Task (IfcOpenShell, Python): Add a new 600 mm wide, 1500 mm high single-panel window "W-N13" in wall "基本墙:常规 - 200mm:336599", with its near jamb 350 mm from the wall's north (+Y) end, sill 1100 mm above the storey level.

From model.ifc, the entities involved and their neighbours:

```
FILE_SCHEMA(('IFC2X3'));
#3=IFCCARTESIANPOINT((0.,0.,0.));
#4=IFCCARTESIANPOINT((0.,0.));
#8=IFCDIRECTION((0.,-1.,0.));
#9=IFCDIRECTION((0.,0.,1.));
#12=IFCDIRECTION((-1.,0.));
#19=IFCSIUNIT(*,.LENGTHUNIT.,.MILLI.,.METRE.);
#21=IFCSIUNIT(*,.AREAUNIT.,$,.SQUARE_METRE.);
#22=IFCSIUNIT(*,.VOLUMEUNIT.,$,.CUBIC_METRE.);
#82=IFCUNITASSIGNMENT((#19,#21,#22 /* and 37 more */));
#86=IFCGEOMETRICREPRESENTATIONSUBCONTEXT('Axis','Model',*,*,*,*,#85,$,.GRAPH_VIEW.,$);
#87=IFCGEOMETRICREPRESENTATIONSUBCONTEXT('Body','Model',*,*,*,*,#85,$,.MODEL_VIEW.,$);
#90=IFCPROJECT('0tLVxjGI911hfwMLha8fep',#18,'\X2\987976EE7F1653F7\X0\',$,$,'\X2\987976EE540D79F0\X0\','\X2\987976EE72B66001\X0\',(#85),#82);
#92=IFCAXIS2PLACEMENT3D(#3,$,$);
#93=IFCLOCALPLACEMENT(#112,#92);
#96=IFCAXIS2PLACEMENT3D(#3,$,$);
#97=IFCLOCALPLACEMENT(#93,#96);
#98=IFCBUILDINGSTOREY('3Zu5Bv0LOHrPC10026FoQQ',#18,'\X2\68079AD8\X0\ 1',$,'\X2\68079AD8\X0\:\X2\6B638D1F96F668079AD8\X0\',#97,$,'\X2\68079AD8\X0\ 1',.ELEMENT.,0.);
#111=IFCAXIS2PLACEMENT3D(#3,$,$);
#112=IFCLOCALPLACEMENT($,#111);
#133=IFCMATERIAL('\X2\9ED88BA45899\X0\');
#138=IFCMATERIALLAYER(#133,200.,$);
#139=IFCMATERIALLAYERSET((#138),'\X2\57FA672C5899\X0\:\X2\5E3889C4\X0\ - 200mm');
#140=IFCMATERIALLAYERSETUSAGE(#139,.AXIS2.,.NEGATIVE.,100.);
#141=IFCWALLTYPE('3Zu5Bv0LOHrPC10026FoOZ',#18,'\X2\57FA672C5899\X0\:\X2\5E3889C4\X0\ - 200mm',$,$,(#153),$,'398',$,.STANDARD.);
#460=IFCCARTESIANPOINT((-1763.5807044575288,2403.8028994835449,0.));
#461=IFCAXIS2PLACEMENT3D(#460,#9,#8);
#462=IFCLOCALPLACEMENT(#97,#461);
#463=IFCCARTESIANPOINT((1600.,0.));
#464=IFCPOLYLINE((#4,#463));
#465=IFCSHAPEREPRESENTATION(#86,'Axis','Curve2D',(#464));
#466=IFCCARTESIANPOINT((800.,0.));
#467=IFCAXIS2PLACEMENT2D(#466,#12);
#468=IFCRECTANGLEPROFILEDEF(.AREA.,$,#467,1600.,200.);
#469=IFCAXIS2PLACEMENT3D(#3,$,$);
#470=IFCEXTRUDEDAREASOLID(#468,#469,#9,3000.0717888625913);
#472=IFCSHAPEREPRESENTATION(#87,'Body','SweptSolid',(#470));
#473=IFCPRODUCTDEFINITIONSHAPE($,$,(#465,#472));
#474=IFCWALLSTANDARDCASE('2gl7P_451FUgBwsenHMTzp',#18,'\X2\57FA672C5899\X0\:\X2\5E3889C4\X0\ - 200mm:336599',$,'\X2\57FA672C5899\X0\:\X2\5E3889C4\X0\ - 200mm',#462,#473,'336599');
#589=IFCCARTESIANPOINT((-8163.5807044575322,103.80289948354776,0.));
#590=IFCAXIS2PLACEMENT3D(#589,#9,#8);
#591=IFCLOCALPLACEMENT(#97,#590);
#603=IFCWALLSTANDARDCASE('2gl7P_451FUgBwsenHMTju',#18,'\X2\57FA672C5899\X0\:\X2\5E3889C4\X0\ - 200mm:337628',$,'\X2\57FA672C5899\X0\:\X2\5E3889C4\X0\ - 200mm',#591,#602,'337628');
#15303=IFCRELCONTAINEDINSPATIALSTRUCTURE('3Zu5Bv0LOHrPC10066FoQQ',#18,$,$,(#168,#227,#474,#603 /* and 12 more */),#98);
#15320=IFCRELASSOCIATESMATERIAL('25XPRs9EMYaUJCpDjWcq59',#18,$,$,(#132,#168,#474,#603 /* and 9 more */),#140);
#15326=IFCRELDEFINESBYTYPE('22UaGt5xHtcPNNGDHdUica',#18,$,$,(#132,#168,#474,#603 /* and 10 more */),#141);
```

```python
import numpy as np
import ifcopenshell
import ifcopenshell.api.feature
import ifcopenshell.api.geometry
import ifcopenshell.api.root
import ifcopenshell.api.spatial
import ifcopenshell.api.type
import ifcopenshell.geom
import ifcopenshell.util.element
import ifcopenshell.util.placement
import ifcopenshell.util.representation
import ifcopenshell.util.shape
import ifcopenshell.util.unit

model = ifcopenshell.open("model.ifc")
unit_scale = ifcopenshell.util.unit.calculate_unit_scale(model)
settings = ifcopenshell.geom.settings()


def volume(element):
    """Net volume in cubic metres, openings subtracted."""
    shape = ifcopenshell.geom.create_shape(settings, element)
    return ifcopenshell.util.shape.get_volume(shape.geometry)


wall = model.by_id(474)
storey = ifcopenshell.util.element.get_container(wall, ifc_class="IfcBuildingStorey")
context = ifcopenshell.util.representation.get_context(model, "Model", "Body", "MODEL_VIEW")
before = volume(wall)

width, height, from_end, sill = 0.6, 1.5, 0.35, 1.1  # metres

# The wall runs along its own X axis, and the end named is its -X end.
wall_shape = ifcopenshell.geom.create_shape(settings, wall)
x, y, z = ifcopenshell.util.shape.get_vertices(wall_shape.geometry).T
start = x.min() + from_end
face, thickness = float(y.min()), float(y.max() - y.min())
wall_matrix = ifcopenshell.util.placement.get_local_placement(wall.ObjectPlacement)
level = ifcopenshell.util.placement.get_local_placement(storey.ObjectPlacement)[2, 3]


def in_wall(x, y):
    """Placement at x, y metres in the wall's axes, at sill height."""
    matrix = wall_matrix.copy()
    matrix[:, 3] = wall_matrix @ np.array([x / unit_scale, y / unit_scale, 0.0, 1.0])
    matrix[2, 3] = level + sill / unit_scale
    return matrix


# Opening: a box that overshoots both wall faces by 50 mm.
opening = ifcopenshell.api.root.create_entity(model, ifc_class="IfcOpeningElement")
box = ifcopenshell.api.geometry.add_wall_representation(
    model, context=context, length=width, height=height, thickness=thickness + 0.1
)
ifcopenshell.api.geometry.assign_representation(model, product=opening, representation=box)
ifcopenshell.api.geometry.edit_object_placement(model, product=opening, matrix=in_wall(start, face - 0.05), is_si=False)
ifcopenshell.api.feature.add_feature(model, feature=opening, element=wall)

window = ifcopenshell.api.root.create_entity(model, ifc_class="IfcWindow", name="W-N13")
window.OverallWidth, window.OverallHeight = width / unit_scale, height / unit_scale
body = ifcopenshell.api.geometry.add_window_representation(
    model,
    context=context,
    overall_width=window.OverallWidth,
    overall_height=window.OverallHeight,
    partition_type="SINGLE_PANEL",
)
ifcopenshell.api.geometry.assign_representation(model, product=window, representation=body)
ifcopenshell.api.spatial.assign_container(model, products=[window], relating_structure=storey)
fills = ifcopenshell.api.feature.add_filling(model, opening=opening, element=window)
fills.OwnerHistory = window.OwnerHistory  # required in IFC2X3

# IFC2X3 keeps the operation on the window style.
style = ifcopenshell.api.root.create_entity(model, ifc_class="IfcWindowStyle", name="W-N13")
style.OperationType, style.ConstructionType = "SINGLE_PANEL", "NOTDEFINED"
style.ParameterTakesPrecedence = style.Sizeable = False
ifcopenshell.api.type.assign_type(model, related_objects=[window], relating_type=style)

# Centre the window in the wall's thickness.
ifcopenshell.api.geometry.edit_object_placement(model, product=window, matrix=in_wall(start, face), is_si=False)
window_shape = ifcopenshell.geom.create_shape(settings, window)
depth = ifcopenshell.util.shape.get_vertices(window_shape.geometry)[:, 1]
offset = face + thickness / 2 - (depth.min() + depth.max()) / 2
ifcopenshell.api.geometry.edit_object_placement(model, product=window, matrix=in_wall(start, offset), is_si=False)

after = volume(wall)

print(f"wall volume {before:.3f} -> {after:.3f} m3")

model.write("model_edited.ifc")
```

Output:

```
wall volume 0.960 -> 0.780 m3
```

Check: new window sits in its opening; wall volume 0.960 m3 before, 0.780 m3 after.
